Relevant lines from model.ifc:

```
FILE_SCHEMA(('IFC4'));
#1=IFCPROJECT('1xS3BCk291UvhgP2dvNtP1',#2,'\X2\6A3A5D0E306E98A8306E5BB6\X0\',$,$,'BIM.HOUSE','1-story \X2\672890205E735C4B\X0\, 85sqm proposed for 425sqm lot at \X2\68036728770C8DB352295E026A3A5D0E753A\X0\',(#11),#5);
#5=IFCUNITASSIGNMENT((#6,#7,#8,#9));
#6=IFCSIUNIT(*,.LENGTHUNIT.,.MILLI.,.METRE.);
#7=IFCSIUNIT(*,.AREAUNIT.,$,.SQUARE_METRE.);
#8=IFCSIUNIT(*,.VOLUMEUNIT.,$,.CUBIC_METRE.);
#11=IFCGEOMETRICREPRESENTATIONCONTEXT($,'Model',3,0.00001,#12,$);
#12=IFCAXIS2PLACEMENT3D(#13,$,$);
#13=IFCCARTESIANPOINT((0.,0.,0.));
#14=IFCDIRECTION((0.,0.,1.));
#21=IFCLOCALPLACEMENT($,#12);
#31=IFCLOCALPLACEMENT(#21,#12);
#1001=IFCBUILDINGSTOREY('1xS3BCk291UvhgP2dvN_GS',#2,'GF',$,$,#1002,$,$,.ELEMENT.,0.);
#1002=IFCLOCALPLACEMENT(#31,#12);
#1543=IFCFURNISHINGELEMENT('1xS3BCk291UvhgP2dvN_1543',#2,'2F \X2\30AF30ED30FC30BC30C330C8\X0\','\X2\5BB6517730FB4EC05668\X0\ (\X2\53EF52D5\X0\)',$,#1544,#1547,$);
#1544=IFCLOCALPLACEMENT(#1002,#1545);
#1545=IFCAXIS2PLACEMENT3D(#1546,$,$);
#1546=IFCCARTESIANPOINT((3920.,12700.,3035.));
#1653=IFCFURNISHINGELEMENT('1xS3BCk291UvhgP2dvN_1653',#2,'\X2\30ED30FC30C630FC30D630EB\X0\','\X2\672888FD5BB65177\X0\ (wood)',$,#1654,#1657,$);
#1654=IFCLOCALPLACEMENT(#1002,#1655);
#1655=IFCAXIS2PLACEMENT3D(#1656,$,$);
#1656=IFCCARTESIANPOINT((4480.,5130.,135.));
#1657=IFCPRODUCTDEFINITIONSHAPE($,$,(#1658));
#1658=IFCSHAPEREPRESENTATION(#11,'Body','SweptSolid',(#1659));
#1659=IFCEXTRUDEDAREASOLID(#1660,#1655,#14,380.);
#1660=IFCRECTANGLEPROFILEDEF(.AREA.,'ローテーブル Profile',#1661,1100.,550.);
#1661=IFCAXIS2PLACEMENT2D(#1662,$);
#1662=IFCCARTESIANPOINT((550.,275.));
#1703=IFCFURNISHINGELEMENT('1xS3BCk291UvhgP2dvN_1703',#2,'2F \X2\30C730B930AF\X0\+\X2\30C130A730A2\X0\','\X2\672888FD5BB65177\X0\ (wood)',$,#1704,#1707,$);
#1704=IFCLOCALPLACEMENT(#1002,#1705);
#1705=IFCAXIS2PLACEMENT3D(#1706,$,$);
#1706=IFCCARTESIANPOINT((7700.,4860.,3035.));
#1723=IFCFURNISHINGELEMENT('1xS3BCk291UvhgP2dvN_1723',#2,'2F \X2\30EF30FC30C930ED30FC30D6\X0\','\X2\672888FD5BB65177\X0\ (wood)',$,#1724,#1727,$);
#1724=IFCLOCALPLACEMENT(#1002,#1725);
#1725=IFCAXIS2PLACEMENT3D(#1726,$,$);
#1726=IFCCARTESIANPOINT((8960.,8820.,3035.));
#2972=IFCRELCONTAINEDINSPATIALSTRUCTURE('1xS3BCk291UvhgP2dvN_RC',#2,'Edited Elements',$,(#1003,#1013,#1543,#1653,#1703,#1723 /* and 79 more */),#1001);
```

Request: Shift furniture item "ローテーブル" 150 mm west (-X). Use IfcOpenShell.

```python
import ifcopenshell
import ifcopenshell.api.geometry
import ifcopenshell.util.placement
import ifcopenshell.util.unit

model = ifcopenshell.open("model.ifc")
unit_scale = ifcopenshell.util.unit.calculate_unit_scale(model)

item = model.by_guid("1xS3BCk291UvhgP2dvN_1653")
matrix = ifcopenshell.util.placement.get_local_placement(item.ObjectPlacement)
matrix[0, 3] -= 0.15 / unit_scale
ifcopenshell.api.geometry.edit_object_placement(model, product=item, matrix=matrix, is_si=False)

print(ifcopenshell.util.placement.get_local_placement(item.ObjectPlacement).round(3) + 0.0)

model.write("model_rev.ifc")
```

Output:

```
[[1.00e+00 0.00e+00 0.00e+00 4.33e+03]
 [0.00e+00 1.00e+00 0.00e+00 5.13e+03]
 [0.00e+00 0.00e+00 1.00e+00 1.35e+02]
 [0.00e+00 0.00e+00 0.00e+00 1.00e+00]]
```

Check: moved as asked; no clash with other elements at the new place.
